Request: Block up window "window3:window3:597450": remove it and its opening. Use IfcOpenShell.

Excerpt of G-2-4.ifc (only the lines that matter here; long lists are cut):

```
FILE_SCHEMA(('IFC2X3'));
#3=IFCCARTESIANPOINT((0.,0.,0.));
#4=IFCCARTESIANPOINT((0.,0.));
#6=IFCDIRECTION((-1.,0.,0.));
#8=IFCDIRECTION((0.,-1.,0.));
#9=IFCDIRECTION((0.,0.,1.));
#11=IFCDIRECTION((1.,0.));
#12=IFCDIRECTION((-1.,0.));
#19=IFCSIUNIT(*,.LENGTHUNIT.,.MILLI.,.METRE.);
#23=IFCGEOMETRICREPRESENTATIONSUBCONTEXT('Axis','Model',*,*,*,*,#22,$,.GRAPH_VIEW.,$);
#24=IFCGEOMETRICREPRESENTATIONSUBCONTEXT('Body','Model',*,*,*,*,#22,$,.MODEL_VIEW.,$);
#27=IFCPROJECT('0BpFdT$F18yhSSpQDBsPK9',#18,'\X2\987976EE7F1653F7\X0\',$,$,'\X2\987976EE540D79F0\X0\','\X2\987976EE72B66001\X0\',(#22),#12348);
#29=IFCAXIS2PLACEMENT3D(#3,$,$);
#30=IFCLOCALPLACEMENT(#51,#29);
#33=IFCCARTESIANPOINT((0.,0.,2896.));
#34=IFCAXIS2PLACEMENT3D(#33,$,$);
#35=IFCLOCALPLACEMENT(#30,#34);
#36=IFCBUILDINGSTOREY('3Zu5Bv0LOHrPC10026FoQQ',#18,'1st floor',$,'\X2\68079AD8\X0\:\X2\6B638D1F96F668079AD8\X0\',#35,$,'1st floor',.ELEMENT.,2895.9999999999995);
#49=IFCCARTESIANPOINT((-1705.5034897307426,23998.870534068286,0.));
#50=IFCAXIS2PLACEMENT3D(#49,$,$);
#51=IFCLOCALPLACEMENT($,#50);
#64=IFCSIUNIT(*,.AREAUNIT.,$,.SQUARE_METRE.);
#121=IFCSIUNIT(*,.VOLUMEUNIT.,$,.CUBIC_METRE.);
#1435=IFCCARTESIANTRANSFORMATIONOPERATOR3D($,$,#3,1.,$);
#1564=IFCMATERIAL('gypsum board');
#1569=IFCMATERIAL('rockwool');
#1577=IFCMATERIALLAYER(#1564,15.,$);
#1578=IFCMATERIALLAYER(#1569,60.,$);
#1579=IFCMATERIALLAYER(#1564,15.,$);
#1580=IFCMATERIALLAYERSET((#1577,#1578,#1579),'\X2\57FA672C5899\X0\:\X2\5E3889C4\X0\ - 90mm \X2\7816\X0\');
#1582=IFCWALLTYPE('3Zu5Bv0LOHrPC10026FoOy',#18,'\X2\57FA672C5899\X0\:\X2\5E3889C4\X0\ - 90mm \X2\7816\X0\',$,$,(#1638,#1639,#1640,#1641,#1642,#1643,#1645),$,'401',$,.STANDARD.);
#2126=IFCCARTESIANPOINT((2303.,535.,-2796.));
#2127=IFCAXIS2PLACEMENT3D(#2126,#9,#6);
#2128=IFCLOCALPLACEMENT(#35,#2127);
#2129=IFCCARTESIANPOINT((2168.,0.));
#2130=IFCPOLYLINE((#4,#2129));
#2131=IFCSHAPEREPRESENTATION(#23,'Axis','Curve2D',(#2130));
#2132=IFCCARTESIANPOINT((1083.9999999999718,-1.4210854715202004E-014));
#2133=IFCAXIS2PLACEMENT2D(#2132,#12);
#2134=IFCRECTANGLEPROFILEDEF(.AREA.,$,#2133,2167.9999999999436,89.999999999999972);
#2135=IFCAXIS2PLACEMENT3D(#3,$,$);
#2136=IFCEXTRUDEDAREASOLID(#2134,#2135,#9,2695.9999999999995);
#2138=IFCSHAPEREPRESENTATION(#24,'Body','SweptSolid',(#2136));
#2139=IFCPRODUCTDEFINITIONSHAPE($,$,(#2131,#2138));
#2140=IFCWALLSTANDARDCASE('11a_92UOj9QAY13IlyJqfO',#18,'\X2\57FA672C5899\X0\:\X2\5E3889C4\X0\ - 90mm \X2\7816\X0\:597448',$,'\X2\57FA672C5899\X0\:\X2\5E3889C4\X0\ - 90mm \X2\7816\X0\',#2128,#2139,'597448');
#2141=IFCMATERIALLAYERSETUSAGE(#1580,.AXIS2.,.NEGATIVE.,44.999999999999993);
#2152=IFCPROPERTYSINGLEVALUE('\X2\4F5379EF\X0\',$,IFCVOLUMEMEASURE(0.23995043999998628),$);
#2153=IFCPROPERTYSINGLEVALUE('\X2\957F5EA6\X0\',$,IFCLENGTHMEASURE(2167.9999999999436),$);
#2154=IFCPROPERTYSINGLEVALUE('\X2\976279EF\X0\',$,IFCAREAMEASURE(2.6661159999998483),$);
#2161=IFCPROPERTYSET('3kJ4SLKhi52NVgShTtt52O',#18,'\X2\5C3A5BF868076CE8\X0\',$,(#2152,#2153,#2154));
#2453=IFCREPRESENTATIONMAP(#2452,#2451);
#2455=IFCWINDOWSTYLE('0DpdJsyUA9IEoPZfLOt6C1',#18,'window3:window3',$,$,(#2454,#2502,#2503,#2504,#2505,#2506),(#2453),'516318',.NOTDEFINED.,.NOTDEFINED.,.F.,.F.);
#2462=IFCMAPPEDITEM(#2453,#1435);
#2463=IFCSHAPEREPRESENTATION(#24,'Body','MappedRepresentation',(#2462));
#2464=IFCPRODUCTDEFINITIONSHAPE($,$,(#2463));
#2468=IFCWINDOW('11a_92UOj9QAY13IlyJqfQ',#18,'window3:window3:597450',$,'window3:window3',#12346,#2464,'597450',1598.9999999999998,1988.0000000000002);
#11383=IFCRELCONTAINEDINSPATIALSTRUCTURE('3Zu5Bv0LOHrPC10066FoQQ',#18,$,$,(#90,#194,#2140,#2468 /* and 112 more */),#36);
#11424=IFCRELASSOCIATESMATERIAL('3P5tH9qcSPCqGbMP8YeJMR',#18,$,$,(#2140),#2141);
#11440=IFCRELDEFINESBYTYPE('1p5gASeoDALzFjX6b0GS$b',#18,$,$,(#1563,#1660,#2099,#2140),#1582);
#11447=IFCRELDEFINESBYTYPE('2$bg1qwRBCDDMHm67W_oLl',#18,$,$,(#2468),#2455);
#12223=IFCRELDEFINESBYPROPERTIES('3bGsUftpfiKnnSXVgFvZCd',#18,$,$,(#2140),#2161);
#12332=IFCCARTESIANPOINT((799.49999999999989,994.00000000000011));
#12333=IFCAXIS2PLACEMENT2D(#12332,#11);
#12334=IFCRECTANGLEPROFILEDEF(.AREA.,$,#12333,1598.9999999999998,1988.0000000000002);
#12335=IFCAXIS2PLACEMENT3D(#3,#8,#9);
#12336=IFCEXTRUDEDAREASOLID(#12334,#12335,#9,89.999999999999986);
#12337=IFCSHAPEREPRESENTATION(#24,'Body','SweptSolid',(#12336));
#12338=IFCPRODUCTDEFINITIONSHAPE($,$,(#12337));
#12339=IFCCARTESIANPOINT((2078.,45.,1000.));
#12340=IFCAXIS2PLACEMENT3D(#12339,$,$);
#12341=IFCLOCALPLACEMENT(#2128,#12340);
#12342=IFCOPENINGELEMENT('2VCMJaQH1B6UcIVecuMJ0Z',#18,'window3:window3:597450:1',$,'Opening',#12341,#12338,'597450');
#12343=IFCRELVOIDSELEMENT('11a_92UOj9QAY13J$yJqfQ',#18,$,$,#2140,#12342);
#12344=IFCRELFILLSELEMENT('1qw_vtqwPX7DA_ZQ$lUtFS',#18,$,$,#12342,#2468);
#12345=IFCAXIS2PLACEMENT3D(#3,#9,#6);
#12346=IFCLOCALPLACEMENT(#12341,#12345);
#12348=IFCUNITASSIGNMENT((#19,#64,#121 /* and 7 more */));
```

```python
import ifcopenshell
import ifcopenshell.api.feature
import ifcopenshell.api.pset
import ifcopenshell.api.root
import ifcopenshell.geom
import ifcopenshell.util.element
import ifcopenshell.util.shape
import ifcopenshell.util.unit

model = ifcopenshell.open("G-2-4.ifc")
area_scale = ifcopenshell.util.unit.calculate_unit_scale(model, "AREAUNIT")
volume_scale = ifcopenshell.util.unit.calculate_unit_scale(model, "VOLUMEUNIT")
settings = ifcopenshell.geom.settings()


def volume(element):
    """Net volume in cubic metres, openings subtracted."""
    shape = ifcopenshell.geom.create_shape(settings, element)
    return ifcopenshell.util.shape.get_volume(shape.geometry)


window = model.by_guid("11a_92UOj9QAY13IlyJqfQ")
opening = window.FillsVoids[0].RelatingOpeningElement
wall = opening.VoidsElements[0].RelatingBuildingElement
before = volume(wall)

ifcopenshell.api.root.remove_product(model, product=window)
ifcopenshell.api.feature.remove_feature(model, feature=opening)

after = volume(wall)
thickness = 0.09  # wall thickness in metres

# Update the wall's stored quantities.
pset = model.by_id(ifcopenshell.util.element.get_pset(wall, "尺寸标注", should_inherit=False)["id"])
ifcopenshell.api.pset.edit_pset(model, pset=pset, properties={
    "体积": model.create_entity("IfcVolumeMeasure", after / volume_scale),
    "面积": model.create_entity("IfcAreaMeasure", after / thickness / area_scale),
})

print(f"wall volume {before:.3f} -> {after:.3f} m3")

model.write("G-2-4_v2.ifc")
```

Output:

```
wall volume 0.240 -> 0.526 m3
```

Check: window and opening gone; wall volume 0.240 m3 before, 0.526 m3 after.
